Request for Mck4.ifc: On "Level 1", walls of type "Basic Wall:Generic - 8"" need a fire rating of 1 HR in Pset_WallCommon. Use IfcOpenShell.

First a look at what the model holds.

```python
import ifcopenshell
import ifcopenshell.util.element

model = ifcopenshell.open("Mck4.ifc")
print(model.schema)
storey = next(s for s in model.by_type("IfcBuildingStorey") if s.Name == "Level 1")
walls = [e for e in ifcopenshell.util.element.get_decomposition(storey) if e.is_a("IfcWall")]
seen = {}
for e in walls:
    element_type = ifcopenshell.util.element.get_type(e)
    key = (element_type.Name if element_type != e and element_type else None, ifcopenshell.util.element.get_pset(e, "Pset_WallCommon", "FireRating"))
    seen[key] = seen.get(key, 0) + 1
for (name, value), count in sorted(seen.items(), key=str):
    print(count, "x", name, "|", value)
```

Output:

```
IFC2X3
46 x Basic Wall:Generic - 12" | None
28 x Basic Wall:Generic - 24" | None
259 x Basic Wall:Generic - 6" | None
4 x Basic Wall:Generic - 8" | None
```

```python
import ifcopenshell
import ifcopenshell.api.pset
import ifcopenshell.util.element

model = ifcopenshell.open("Mck4.ifc")

storey = next(s for s in model.by_type("IfcBuildingStorey") if s.Name == "Level 1")
walls = [e for e in ifcopenshell.util.element.get_decomposition(storey) if e.is_a("IfcWall")]

count = 0
for e in walls:
    element_type = ifcopenshell.util.element.get_type(e)
    if element_type in (None, e) or element_type.Name != 'Basic Wall:Generic - 8"':
        continue
    # add_pset returns the element's existing set when there is one.
    pset = ifcopenshell.api.pset.add_pset(model, product=e, name="Pset_WallCommon")
    ifcopenshell.api.pset.edit_pset(model, pset=pset, properties={"FireRating": "1 HR"})
    count += 1

print(count, "walls updated")

model.write("Mck4_rev.ifc")
```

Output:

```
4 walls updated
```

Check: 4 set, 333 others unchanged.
